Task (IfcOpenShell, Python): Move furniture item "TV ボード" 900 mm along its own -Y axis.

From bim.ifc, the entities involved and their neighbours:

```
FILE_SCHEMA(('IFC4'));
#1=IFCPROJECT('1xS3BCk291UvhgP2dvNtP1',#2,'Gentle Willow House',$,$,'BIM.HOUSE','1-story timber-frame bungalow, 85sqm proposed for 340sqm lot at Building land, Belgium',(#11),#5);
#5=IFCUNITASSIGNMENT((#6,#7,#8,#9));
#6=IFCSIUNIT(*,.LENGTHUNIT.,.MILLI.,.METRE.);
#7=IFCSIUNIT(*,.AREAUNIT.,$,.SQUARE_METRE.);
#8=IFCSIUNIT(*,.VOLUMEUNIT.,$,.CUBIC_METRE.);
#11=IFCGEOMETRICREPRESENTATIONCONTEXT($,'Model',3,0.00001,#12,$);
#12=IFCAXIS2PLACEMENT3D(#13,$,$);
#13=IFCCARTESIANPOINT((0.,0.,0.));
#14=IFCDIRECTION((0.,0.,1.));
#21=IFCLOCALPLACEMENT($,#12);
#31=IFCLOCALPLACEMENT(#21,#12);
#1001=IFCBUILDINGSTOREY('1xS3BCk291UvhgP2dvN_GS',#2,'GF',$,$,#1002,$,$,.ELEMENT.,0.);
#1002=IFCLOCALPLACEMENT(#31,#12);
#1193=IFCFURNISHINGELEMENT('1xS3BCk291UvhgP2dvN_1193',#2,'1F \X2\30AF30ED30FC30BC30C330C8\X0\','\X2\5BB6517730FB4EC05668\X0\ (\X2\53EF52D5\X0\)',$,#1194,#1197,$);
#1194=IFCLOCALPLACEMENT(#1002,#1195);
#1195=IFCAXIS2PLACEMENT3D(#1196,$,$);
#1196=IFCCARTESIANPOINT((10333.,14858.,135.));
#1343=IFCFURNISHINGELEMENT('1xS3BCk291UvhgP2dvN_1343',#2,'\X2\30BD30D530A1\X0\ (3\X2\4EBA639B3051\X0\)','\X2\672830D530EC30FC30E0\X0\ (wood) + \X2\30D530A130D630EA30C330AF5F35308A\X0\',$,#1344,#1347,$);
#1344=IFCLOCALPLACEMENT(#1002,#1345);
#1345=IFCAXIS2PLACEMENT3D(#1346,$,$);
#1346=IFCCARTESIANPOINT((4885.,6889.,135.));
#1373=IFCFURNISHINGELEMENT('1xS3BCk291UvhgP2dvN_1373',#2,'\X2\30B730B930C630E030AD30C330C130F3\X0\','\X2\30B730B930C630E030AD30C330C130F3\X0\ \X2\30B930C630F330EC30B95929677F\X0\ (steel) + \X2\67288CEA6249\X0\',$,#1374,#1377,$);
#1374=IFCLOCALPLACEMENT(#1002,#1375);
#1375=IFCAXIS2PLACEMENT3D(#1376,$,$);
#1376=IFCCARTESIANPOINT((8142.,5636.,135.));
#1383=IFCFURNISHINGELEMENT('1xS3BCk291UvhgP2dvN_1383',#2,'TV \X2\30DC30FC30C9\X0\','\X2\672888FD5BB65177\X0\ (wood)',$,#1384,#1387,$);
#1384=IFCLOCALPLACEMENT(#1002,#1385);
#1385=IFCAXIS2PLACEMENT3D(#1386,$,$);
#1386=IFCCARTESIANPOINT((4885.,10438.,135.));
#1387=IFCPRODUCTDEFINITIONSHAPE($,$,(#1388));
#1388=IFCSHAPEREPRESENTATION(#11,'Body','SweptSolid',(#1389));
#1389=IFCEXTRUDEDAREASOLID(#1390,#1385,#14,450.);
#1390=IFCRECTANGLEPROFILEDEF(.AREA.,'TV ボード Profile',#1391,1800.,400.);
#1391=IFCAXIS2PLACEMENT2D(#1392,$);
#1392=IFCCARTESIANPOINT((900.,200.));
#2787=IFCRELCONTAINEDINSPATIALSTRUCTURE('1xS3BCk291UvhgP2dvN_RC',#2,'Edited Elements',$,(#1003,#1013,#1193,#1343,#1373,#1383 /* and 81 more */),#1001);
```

```python
import ifcopenshell
import ifcopenshell.api.geometry
import ifcopenshell.util.placement
import ifcopenshell.util.unit

model = ifcopenshell.open("bim.ifc")
unit_scale = ifcopenshell.util.unit.calculate_unit_scale(model)

item = model.by_guid("1xS3BCk291UvhgP2dvN_1383")
matrix = ifcopenshell.util.placement.get_local_placement(item.ObjectPlacement)
matrix[:3, 3] -= matrix[:3, 1] * 0.9 / unit_scale
ifcopenshell.api.geometry.edit_object_placement(model, product=item, matrix=matrix, is_si=False)

print(ifcopenshell.util.placement.get_local_placement(item.ObjectPlacement).round(3) + 0.0)

model.write("bim_v2.ifc")
```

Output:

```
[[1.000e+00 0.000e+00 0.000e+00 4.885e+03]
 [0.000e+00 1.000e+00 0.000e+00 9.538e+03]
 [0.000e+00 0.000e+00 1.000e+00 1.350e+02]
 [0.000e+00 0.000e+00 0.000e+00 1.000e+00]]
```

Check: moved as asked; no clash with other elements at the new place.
